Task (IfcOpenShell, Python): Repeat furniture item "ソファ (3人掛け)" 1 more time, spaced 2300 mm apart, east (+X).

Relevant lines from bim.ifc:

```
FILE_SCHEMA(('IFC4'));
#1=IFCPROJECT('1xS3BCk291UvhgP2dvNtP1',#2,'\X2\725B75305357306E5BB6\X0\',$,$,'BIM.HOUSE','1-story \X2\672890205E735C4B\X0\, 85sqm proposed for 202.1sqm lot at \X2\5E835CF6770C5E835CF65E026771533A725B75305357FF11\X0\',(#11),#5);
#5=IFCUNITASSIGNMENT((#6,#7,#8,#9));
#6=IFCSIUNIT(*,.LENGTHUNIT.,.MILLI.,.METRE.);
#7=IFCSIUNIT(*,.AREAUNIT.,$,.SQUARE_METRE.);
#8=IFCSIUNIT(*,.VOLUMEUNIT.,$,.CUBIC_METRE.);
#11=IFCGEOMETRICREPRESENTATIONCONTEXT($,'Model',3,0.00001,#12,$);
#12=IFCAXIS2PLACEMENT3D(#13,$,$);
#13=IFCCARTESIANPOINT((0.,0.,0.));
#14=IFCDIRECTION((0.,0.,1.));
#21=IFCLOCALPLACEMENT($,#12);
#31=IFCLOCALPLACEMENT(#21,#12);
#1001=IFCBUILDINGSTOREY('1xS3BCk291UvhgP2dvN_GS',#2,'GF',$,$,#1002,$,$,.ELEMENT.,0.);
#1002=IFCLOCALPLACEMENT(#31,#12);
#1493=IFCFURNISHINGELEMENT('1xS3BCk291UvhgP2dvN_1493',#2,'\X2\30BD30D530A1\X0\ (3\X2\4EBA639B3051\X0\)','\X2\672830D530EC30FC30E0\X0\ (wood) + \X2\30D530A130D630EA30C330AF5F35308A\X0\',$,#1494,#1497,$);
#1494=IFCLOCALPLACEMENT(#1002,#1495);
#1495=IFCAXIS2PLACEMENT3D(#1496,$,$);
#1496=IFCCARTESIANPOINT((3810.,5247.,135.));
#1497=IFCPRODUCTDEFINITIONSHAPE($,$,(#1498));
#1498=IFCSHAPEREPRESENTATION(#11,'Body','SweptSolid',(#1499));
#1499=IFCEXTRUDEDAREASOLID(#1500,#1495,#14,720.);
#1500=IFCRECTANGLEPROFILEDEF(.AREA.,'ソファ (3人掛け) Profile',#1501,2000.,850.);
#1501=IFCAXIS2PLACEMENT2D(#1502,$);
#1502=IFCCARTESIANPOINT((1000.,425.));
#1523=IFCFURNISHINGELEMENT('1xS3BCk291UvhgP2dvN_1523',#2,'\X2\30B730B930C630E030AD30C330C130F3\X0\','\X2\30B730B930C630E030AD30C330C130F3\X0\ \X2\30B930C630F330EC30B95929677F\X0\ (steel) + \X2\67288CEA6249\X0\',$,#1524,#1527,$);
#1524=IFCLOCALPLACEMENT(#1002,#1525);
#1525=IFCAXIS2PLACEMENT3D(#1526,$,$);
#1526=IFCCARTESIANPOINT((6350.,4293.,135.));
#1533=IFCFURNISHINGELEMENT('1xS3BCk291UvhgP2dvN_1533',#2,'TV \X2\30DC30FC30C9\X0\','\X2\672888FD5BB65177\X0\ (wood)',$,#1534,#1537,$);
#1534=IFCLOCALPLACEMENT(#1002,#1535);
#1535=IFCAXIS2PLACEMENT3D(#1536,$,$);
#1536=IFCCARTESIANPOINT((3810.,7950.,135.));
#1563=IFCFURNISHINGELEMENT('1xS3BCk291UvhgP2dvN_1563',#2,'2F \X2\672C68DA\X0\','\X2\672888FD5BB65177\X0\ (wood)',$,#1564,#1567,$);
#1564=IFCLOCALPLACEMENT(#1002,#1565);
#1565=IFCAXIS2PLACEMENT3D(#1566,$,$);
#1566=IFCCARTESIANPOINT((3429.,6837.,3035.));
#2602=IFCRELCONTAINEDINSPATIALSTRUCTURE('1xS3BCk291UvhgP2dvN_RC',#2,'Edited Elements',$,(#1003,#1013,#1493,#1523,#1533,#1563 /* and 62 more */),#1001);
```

```python
import numpy as np
import ifcopenshell
import ifcopenshell.api.geometry
import ifcopenshell.api.root
import ifcopenshell.util.element
import ifcopenshell.util.placement
import ifcopenshell.util.unit

model = ifcopenshell.open("bim.ifc")
unit_scale = ifcopenshell.util.unit.calculate_unit_scale(model)


def reuse_history(source, copy):
    """copy_class also copies each property set's owner history, people and application; keep the originals."""
    for rel in copy.IsDefinedBy:
        if rel.is_a("IfcRelDefinesByProperties") and (history := rel.RelatingPropertyDefinition.OwnerHistory):
            rel.RelatingPropertyDefinition.OwnerHistory = source.OwnerHistory
            ifcopenshell.util.element.remove_deep2(model, history)


source = model.by_guid("1xS3BCk291UvhgP2dvN_1493")
base = ifcopenshell.util.placement.get_local_placement(source.ObjectPlacement)
step = np.array([1.0, 0.0, 0.0]) * 2.3 / unit_scale

for i in range(1, 2):
    copy = ifcopenshell.api.root.copy_class(model, product=source)
    copy.Representation = ifcopenshell.util.element.copy_deep(
        model, source.Representation, exclude=["IfcGeometricRepresentationContext", "IfcRepresentationMap"]
    )
    reuse_history(source, copy)
    matrix = base.copy()
    matrix[:3, 3] += i * step
    print("added at", matrix[:3, 3].round(3) + 0.0)
    ifcopenshell.api.geometry.edit_object_placement(model, product=copy, matrix=matrix, is_si=False)

model.write("bim_v2.ifc")
```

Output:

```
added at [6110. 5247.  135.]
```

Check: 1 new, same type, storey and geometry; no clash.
